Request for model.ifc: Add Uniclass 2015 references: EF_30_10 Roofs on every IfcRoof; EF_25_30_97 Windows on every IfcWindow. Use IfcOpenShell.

First a look at what the model holds.

```python
import ifcopenshell

model = ifcopenshell.open("model.ifc")
print(model.schema)
print("classifications:", [c.Name for c in model.by_type("IfcClassification")])
for ifc_class in ("IfcDoor", "IfcRoof", "IfcStair", "IfcWall", "IfcWindow"):
    print(ifc_class, len(model.by_type(ifc_class)))
```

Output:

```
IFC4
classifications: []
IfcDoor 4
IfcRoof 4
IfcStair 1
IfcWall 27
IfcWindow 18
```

```python
import ifcopenshell
import ifcopenshell.api.classification

model = ifcopenshell.open("model.ifc")

system = ifcopenshell.api.classification.add_classification(model, classification="Uniclass 2015")

codes = {
    "IfcRoof": ("EF_30_10", "Roofs"),
    "IfcWindow": ("EF_25_30_97", "Windows"),
}
for ifc_class, (code, name) in codes.items():
    products = model.by_type(ifc_class)
    ifcopenshell.api.classification.add_reference(
        model, products=products, classification=system, identification=code, name=name
    )
    print(code, len(products))

model.write("model_edited.ifc")
```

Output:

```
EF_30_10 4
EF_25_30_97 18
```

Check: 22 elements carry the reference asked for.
